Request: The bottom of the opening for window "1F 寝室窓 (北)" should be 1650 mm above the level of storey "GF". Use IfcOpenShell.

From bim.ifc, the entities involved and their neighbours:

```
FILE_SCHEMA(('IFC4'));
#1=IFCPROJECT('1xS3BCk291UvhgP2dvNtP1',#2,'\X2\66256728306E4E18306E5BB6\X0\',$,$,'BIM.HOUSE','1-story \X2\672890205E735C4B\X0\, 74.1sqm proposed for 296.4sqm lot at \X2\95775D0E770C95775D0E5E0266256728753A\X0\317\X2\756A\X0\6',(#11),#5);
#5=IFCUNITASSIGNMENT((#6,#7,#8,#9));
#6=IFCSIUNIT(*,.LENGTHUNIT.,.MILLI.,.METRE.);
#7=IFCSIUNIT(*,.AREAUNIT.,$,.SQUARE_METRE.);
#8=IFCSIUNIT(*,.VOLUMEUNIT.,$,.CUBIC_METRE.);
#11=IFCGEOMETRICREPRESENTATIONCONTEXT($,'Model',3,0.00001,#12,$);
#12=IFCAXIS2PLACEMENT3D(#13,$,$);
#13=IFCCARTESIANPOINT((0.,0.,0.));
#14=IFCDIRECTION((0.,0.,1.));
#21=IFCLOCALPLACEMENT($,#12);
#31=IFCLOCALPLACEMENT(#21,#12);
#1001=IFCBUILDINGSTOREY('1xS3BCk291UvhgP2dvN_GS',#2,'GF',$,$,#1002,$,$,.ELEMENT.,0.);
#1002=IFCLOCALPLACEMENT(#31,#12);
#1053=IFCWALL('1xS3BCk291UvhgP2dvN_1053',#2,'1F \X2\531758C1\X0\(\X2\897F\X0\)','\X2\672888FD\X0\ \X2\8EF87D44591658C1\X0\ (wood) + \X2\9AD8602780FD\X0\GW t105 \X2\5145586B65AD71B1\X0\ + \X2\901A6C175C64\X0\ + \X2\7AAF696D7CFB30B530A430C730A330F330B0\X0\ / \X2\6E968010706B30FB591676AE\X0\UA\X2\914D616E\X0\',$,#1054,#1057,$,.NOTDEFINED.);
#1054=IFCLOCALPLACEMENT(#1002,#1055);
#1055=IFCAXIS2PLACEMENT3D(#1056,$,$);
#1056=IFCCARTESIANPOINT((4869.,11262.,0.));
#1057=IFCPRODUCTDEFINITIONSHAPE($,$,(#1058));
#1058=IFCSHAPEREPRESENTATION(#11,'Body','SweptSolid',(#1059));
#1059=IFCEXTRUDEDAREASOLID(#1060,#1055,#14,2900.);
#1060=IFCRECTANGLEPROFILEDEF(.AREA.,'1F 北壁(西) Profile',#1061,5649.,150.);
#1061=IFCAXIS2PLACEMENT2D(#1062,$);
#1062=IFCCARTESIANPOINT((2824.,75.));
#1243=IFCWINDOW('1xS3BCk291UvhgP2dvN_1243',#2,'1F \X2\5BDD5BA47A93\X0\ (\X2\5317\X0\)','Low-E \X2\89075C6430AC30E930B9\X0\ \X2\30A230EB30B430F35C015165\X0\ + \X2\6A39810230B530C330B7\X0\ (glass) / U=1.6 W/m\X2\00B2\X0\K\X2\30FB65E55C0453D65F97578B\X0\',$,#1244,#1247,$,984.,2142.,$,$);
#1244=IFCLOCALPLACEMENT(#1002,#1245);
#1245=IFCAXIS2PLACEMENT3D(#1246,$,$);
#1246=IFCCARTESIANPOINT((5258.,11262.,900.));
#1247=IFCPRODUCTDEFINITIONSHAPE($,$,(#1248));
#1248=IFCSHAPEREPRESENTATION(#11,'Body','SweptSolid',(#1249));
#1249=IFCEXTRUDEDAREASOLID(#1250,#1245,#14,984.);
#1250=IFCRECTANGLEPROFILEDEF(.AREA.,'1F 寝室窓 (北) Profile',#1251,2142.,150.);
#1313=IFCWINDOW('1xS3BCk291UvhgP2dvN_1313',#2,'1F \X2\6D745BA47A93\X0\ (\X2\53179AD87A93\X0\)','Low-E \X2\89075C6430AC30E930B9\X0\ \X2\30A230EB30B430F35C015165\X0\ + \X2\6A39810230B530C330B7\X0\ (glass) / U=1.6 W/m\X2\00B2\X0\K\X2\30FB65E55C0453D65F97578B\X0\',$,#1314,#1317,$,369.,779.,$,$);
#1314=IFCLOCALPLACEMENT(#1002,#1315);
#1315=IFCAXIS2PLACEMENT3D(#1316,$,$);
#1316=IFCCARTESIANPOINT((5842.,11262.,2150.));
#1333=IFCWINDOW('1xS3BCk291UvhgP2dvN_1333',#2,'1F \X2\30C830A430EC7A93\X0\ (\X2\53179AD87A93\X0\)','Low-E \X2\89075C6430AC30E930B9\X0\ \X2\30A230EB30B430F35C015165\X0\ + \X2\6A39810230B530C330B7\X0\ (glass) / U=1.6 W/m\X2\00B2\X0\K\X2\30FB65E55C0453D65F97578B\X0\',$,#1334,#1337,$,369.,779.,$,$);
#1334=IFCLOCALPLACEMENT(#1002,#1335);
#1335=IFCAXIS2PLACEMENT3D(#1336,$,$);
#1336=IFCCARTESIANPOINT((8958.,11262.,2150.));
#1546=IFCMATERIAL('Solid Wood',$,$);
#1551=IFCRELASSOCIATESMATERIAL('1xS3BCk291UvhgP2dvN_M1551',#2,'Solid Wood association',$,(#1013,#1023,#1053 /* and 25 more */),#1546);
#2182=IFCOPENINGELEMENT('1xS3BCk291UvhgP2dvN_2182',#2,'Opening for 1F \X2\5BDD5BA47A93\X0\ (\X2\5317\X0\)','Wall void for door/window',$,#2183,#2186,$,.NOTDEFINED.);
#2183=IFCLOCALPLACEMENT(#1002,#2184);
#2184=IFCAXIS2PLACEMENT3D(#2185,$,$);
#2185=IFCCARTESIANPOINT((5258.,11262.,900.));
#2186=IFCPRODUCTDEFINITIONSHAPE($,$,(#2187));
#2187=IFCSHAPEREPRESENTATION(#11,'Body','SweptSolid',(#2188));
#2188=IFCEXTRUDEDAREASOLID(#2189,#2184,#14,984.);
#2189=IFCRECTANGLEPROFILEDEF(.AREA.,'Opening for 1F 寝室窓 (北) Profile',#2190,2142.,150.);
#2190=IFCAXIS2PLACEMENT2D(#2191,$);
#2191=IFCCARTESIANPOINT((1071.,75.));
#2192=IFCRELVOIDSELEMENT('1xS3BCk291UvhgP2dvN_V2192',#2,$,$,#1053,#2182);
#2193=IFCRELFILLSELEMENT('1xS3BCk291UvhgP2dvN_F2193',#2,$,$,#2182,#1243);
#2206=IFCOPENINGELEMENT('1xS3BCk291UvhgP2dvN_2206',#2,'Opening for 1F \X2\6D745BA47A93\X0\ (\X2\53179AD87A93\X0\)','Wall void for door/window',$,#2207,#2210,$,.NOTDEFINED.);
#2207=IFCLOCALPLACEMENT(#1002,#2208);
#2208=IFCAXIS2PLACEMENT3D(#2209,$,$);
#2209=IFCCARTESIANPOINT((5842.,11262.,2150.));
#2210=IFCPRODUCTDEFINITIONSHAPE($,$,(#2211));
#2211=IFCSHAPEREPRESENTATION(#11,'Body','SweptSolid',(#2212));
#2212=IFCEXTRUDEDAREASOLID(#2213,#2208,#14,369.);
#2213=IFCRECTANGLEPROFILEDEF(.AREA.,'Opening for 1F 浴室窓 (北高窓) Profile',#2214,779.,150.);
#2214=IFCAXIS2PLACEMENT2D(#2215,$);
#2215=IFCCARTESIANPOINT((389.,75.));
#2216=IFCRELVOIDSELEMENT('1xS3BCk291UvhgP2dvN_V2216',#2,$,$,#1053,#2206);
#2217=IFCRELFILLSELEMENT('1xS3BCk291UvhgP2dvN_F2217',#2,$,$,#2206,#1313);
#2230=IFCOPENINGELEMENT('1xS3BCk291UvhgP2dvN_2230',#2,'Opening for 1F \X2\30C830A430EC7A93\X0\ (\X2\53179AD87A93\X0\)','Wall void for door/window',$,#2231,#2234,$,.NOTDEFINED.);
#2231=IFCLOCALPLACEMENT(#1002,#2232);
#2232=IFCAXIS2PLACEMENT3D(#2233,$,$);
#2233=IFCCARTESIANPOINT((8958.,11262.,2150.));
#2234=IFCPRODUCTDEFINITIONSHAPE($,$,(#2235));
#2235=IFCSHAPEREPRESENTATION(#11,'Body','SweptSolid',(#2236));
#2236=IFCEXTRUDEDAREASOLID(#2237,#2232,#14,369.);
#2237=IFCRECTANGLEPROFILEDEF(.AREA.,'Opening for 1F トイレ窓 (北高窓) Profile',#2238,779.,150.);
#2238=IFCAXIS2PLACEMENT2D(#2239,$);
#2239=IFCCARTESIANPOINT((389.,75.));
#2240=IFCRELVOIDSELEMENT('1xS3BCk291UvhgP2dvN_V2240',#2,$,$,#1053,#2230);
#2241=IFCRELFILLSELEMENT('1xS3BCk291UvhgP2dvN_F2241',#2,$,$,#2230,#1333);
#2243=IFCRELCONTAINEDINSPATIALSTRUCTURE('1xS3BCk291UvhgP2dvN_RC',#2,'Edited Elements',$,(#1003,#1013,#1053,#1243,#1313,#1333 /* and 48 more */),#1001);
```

```python
import numpy as np
import ifcopenshell
import ifcopenshell.api.geometry
import ifcopenshell.geom
import ifcopenshell.util.element
import ifcopenshell.util.placement
import ifcopenshell.util.shape
import ifcopenshell.util.unit

model = ifcopenshell.open("bim.ifc")
unit_scale = ifcopenshell.util.unit.calculate_unit_scale(model)

window = model.by_id(1243)
opening = window.FillsVoids[0].RelatingOpeningElement
storey = ifcopenshell.util.element.get_container(window, ifc_class="IfcBuildingStorey")
level = ifcopenshell.util.placement.get_local_placement(storey.ObjectPlacement)[2, 3]

# The opening's origin need not be at the sill, so measure its lowest point.
shape = ifcopenshell.geom.create_shape(ifcopenshell.geom.settings(), opening)
bottom = ifcopenshell.util.shape.get_shape_bottom_elevation(shape, shape.geometry) / unit_scale
dz = level + 1650.0 - bottom

shift = np.array([0.0, 0.0, dz])
# The window is not placed relative to its opening, so move both.
for product in (opening, window):
    matrix = ifcopenshell.util.placement.get_local_placement(product.ObjectPlacement)
    matrix[:3, 3] += shift
    ifcopenshell.api.geometry.edit_object_placement(model, product=product, matrix=matrix, is_si=False)

print(f"moved by {dz * unit_scale:+.3f} m")

model.write("bim_v2.ifc")
```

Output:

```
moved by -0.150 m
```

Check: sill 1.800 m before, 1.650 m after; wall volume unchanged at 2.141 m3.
